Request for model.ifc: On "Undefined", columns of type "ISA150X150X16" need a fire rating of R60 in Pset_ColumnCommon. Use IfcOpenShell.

First a look at what the model holds.

```python
import ifcopenshell
import ifcopenshell.util.element

model = ifcopenshell.open("model.ifc")
print(model.schema)
storey = next(s for s in model.by_type("IfcBuildingStorey") if s.Name == "Undefined")
columns = [e for e in ifcopenshell.util.element.get_decomposition(storey) if e.is_a("IfcColumn")]
seen = {}
for e in columns:
    element_type = ifcopenshell.util.element.get_type(e)
    key = (element_type.Name if element_type != e and element_type else None, ifcopenshell.util.element.get_pset(e, "Pset_ColumnCommon", "FireRating"))
    seen[key] = seen.get(key, 0) + 1
for (name, value), count in sorted(seen.items(), key=str):
    print(count, "x", name, "|", value)
```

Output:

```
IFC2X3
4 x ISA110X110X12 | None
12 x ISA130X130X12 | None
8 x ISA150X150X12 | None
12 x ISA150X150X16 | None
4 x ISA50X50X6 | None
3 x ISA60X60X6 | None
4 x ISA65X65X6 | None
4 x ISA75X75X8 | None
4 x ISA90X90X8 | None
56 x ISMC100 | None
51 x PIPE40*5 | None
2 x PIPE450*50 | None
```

```python
import ifcopenshell
import ifcopenshell.api.pset
import ifcopenshell.util.element

model = ifcopenshell.open("model.ifc")

storey = next(s for s in model.by_type("IfcBuildingStorey") if s.Name == "Undefined")
columns = [e for e in ifcopenshell.util.element.get_decomposition(storey) if e.is_a("IfcColumn")]

count = 0
for e in columns:
    element_type = ifcopenshell.util.element.get_type(e)
    if element_type in (None, e) or element_type.Name != "ISA150X150X16":
        continue
    found = ifcopenshell.util.element.get_pset(e, "Pset_ColumnCommon", should_inherit=False)
    if found:
        pset = model.by_id(found["id"])
        if len(ifcopenshell.util.element.get_elements_by_pset(pset)) > 1:
            pset = ifcopenshell.api.pset.unshare_pset(model, products=[e], pset=pset)[0]
    else:
        pset = ifcopenshell.api.pset.add_pset(model, product=e, name="Pset_ColumnCommon")
    ifcopenshell.api.pset.edit_pset(model, pset=pset, properties={"FireRating": "R60"})
    count += 1

print(count, "columns updated")

model.write("model_v2.ifc")
```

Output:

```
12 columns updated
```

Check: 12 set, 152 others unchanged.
